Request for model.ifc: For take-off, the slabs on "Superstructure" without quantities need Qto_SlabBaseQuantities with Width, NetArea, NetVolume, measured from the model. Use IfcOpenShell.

First a look at what the model holds.

```python
import ifcopenshell
import ifcopenshell.util.element
import ifcopenshell.util.unit

model = ifcopenshell.open("model.ifc")
print(model.schema)
for unit_type in ("LENGTHUNIT", "AREAUNIT", "VOLUMEUNIT"):
    print(unit_type, ifcopenshell.util.unit.calculate_unit_scale(model, unit_type))
storey = next(s for s in model.by_type("IfcBuildingStorey") if s.Name == "Superstructure")
slabs = [e for e in ifcopenshell.util.element.get_decomposition(storey) if e.is_a("IfcSlab")]
for e in sorted(slabs, key=lambda e: e.id()):
    print(e.id(), e.is_a(), e.Name, list(ifcopenshell.util.element.get_psets(e, qtos_only=True)), sep=" | ")
```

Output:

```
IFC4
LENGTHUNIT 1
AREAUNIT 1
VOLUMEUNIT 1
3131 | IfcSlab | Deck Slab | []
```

```python
import ifcopenshell
import ifcopenshell.api.pset
import ifcopenshell.geom
import ifcopenshell.util.element
import ifcopenshell.util.shape
import ifcopenshell.util.unit

model = ifcopenshell.open("model.ifc")
unit_scale = ifcopenshell.util.unit.calculate_unit_scale(model)
area_scale = ifcopenshell.util.unit.calculate_unit_scale(model, "AREAUNIT")
volume_scale = ifcopenshell.util.unit.calculate_unit_scale(model, "VOLUMEUNIT")
settings = ifcopenshell.geom.settings()

storey = next(s for s in model.by_type("IfcBuildingStorey") if s.Name == "Superstructure")
slabs = [e for e in ifcopenshell.util.element.get_decomposition(storey) if e.is_a("IfcSlab")]

for e in sorted(slabs, key=lambda e: e.id()):
    if ifcopenshell.util.element.get_psets(e, qtos_only=True, should_inherit=False):
        continue
    # Geometry comes back in metres, in the element's own axes.
    shape = ifcopenshell.geom.create_shape(settings, e)
    values = {
        "Width": ifcopenshell.util.shape.get_z(shape.geometry) / unit_scale,
        "NetArea": ifcopenshell.util.shape.get_footprint_area(shape.geometry) / area_scale,
        "NetVolume": ifcopenshell.util.shape.get_volume(shape.geometry) / volume_scale,
    }
    qto = ifcopenshell.api.pset.add_qto(model, product=e, name="Qto_SlabBaseQuantities")
    ifcopenshell.api.pset.edit_qto(model, qto=qto, properties=values)
    print(e.id(), {k: round(v, 3) for k, v in values.items()})

model.write("model_v2.ifc")
```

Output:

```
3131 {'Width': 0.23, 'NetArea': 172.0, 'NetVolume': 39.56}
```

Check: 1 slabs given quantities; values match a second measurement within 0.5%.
